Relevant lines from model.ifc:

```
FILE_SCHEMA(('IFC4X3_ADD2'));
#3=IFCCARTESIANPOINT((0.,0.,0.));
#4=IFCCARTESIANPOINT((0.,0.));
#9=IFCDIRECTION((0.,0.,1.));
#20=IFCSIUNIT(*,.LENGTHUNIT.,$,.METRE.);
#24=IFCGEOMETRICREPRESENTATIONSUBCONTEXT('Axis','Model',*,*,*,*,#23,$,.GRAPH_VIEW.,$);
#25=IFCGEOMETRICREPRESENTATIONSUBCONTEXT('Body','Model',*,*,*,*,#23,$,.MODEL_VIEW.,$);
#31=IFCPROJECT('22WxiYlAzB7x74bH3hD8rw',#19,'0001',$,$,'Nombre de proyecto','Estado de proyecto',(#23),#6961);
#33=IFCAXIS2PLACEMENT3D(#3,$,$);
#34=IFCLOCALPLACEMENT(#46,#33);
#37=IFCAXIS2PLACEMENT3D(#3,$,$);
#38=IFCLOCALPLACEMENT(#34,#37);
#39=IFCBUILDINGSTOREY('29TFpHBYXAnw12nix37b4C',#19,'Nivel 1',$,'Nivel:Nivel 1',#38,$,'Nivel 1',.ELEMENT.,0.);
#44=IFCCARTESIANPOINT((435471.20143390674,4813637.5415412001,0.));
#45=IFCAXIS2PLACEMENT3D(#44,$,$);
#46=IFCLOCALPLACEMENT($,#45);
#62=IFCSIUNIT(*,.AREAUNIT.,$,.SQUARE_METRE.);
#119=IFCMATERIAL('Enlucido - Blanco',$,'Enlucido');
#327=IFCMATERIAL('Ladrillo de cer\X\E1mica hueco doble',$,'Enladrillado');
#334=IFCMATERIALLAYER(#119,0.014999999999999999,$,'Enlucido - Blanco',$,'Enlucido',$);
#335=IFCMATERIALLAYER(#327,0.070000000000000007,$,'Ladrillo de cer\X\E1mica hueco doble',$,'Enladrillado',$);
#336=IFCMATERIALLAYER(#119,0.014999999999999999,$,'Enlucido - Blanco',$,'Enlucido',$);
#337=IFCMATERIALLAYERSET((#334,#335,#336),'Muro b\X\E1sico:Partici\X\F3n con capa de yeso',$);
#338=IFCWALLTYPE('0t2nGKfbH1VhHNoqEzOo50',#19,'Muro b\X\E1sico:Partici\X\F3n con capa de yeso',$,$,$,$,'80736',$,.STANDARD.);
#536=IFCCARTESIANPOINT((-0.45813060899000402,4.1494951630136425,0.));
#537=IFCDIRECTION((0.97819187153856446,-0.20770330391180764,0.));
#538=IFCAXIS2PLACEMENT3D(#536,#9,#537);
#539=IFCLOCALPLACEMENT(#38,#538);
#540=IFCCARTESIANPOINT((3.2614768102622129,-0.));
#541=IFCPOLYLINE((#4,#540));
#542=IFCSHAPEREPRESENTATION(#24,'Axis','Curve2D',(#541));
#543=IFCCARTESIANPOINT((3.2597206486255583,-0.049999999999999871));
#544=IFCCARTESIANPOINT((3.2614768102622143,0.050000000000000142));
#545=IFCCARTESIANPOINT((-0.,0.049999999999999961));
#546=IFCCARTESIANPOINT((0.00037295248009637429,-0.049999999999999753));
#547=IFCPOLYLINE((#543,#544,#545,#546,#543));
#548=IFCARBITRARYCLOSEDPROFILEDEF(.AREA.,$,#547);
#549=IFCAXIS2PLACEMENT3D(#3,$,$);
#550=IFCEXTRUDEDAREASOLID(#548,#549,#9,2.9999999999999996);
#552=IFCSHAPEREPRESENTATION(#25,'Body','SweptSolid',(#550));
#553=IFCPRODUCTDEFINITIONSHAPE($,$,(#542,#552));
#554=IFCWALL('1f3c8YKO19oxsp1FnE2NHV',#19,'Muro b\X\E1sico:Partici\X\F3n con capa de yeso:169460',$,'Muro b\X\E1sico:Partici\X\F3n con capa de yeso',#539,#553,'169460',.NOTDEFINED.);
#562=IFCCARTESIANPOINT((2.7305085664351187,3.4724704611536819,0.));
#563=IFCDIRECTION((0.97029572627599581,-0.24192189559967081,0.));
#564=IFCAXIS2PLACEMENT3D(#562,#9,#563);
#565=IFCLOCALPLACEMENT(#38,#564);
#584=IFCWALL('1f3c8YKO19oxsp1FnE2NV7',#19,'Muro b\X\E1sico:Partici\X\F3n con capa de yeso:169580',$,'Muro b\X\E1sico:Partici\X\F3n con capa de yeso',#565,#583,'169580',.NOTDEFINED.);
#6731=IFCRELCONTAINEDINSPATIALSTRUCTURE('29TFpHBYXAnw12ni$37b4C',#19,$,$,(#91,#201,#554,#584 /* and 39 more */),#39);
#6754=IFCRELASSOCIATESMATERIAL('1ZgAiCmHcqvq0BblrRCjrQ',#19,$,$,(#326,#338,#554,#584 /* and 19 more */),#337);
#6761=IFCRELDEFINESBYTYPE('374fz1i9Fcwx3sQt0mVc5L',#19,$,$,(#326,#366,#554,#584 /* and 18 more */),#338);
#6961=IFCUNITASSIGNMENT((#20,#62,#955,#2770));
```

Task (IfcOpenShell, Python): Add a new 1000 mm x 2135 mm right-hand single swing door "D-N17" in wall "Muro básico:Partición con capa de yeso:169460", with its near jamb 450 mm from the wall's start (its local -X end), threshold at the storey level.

```python
import numpy as np
import ifcopenshell
import ifcopenshell.api.feature
import ifcopenshell.api.geometry
import ifcopenshell.api.root
import ifcopenshell.api.spatial
import ifcopenshell.geom
import ifcopenshell.util.element
import ifcopenshell.util.placement
import ifcopenshell.util.representation
import ifcopenshell.util.shape
import ifcopenshell.util.unit

model = ifcopenshell.open("model.ifc")
unit_scale = ifcopenshell.util.unit.calculate_unit_scale(model)
settings = ifcopenshell.geom.settings()


def volume(element):
    """Net volume in cubic metres, openings subtracted."""
    shape = ifcopenshell.geom.create_shape(settings, element)
    return ifcopenshell.util.shape.get_volume(shape.geometry)


wall = model.by_guid("1f3c8YKO19oxsp1FnE2NHV")
storey = ifcopenshell.util.element.get_container(wall, ifc_class="IfcBuildingStorey")
context = ifcopenshell.util.representation.get_context(model, "Model", "Body", "MODEL_VIEW")
before = volume(wall)

width, height, from_end, sill = 1, 2.135, 0.45, 0.0  # metres

# The wall runs along its own X axis, and the end named is its -X end.
wall_shape = ifcopenshell.geom.create_shape(settings, wall)
x, y, z = ifcopenshell.util.shape.get_vertices(wall_shape.geometry).T
start = x.min() + from_end
face, thickness = float(y.min()), float(y.max() - y.min())
wall_matrix = ifcopenshell.util.placement.get_local_placement(wall.ObjectPlacement)
level = ifcopenshell.util.placement.get_local_placement(storey.ObjectPlacement)[2, 3]


def in_wall(x, y):
    """Placement at x, y metres in the wall's axes, at sill height."""
    matrix = wall_matrix.copy()
    matrix[:, 3] = wall_matrix @ np.array([x / unit_scale, y / unit_scale, 0.0, 1.0])
    matrix[2, 3] = level + sill / unit_scale
    return matrix


# Opening: a box that overshoots both wall faces by 50 mm.
opening = ifcopenshell.api.root.create_entity(model, ifc_class="IfcOpeningElement", predefined_type="OPENING")
box = ifcopenshell.api.geometry.add_wall_representation(
    model, context=context, length=width, height=height, thickness=thickness + 0.1
)
ifcopenshell.api.geometry.assign_representation(model, product=opening, representation=box)
ifcopenshell.api.geometry.edit_object_placement(model, product=opening, matrix=in_wall(start, face - 0.05), is_si=False)
ifcopenshell.api.feature.add_feature(model, feature=opening, element=wall)

door = ifcopenshell.api.root.create_entity(model, ifc_class="IfcDoor", name="D-N17", predefined_type="DOOR")
door.OverallWidth, door.OverallHeight = width / unit_scale, height / unit_scale
door.OperationType = "SINGLE_SWING_RIGHT"
body = ifcopenshell.api.geometry.add_door_representation(
    model,
    context=context,
    overall_width=door.OverallWidth,
    overall_height=door.OverallHeight,
    operation_type="SINGLE_SWING_RIGHT",
    lining_properties={"LiningDepth": thickness / unit_scale, "ThresholdDepth": thickness / unit_scale},
)
ifcopenshell.api.geometry.assign_representation(model, product=door, representation=body)
ifcopenshell.api.spatial.assign_container(model, products=[door], relating_structure=storey)
ifcopenshell.api.feature.add_filling(model, opening=opening, element=door)

# The lining spans the wall, so the door starts at the wall face.
ifcopenshell.api.geometry.edit_object_placement(model, product=door, matrix=in_wall(start, face), is_si=False)

after = volume(wall)

print(f"wall volume {before:.3f} -> {after:.3f} m3")

model.write("model_rev.ifc")
```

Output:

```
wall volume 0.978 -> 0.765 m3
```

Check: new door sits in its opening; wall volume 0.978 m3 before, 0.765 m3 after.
